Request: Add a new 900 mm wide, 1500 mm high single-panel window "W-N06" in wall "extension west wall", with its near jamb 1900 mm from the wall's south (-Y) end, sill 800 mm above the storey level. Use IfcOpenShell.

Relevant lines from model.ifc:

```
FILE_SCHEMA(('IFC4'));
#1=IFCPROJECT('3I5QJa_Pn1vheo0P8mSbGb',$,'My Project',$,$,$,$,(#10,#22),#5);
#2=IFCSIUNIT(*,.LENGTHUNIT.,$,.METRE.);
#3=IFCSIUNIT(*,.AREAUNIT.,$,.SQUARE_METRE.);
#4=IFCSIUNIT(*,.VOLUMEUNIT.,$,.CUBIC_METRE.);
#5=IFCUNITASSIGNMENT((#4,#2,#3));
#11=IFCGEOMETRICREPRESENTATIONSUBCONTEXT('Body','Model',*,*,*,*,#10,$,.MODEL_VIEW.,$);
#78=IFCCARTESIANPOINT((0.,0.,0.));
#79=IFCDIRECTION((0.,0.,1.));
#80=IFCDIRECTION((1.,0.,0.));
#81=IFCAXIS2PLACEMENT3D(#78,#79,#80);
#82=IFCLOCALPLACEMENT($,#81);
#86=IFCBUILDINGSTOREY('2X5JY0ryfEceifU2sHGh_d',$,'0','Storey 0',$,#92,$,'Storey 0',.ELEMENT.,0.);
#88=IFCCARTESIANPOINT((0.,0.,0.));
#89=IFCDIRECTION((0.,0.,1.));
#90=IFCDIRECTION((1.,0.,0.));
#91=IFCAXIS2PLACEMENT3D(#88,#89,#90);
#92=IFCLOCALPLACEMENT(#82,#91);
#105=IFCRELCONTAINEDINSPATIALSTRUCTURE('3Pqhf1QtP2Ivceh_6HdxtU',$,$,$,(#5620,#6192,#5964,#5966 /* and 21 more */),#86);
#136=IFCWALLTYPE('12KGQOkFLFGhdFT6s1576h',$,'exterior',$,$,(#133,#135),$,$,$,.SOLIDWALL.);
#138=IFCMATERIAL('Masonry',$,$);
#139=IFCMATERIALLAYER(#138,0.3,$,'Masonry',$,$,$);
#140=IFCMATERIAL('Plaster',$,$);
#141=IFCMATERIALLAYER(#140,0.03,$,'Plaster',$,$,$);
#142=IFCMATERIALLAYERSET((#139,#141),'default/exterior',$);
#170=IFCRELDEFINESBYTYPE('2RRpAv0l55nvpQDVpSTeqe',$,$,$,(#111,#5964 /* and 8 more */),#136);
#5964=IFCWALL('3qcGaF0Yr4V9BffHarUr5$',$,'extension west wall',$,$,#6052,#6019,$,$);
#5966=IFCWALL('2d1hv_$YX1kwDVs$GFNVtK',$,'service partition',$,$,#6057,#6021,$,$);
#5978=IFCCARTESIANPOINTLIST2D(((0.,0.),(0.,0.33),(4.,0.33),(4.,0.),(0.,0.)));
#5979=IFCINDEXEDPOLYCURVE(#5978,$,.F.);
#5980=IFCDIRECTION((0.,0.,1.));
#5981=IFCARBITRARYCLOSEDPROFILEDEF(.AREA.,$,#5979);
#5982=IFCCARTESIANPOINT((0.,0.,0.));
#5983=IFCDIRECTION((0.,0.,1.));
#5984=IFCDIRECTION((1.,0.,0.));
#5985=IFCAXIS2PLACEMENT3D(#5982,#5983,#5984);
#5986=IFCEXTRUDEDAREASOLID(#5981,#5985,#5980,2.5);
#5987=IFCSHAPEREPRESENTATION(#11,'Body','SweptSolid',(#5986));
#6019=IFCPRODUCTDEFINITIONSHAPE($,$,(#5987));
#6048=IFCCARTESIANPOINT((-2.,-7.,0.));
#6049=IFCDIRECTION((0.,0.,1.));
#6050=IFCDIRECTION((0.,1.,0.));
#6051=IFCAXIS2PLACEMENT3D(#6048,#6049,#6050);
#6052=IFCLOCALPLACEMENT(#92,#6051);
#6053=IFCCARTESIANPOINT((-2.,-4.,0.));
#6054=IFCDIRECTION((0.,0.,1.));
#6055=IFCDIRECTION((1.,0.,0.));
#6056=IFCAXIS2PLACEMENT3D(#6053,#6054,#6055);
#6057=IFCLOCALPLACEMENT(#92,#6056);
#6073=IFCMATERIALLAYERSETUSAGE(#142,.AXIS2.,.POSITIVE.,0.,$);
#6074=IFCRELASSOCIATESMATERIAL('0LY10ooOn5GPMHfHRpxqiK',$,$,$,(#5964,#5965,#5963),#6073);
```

```python
import numpy as np
import ifcopenshell
import ifcopenshell.api.feature
import ifcopenshell.api.geometry
import ifcopenshell.api.root
import ifcopenshell.api.spatial
import ifcopenshell.geom
import ifcopenshell.util.element
import ifcopenshell.util.placement
import ifcopenshell.util.representation
import ifcopenshell.util.shape
import ifcopenshell.util.unit

model = ifcopenshell.open("model.ifc")
unit_scale = ifcopenshell.util.unit.calculate_unit_scale(model)
settings = ifcopenshell.geom.settings()


def volume(element):
    """Net volume in cubic metres, openings subtracted."""
    shape = ifcopenshell.geom.create_shape(settings, element)
    return ifcopenshell.util.shape.get_volume(shape.geometry)


wall = model.by_guid("3qcGaF0Yr4V9BffHarUr5$")
storey = ifcopenshell.util.element.get_container(wall, ifc_class="IfcBuildingStorey")
context = ifcopenshell.util.representation.get_context(model, "Model", "Body", "MODEL_VIEW")
before = volume(wall)

width, height, from_end, sill = 0.9, 1.5, 1.9, 0.8  # metres

# The wall runs along its own X axis, and the end named is its -X end.
wall_shape = ifcopenshell.geom.create_shape(settings, wall)
x, y, z = ifcopenshell.util.shape.get_vertices(wall_shape.geometry).T
start = x.min() + from_end
face, thickness = float(y.min()), float(y.max() - y.min())
wall_matrix = ifcopenshell.util.placement.get_local_placement(wall.ObjectPlacement)
level = ifcopenshell.util.placement.get_local_placement(storey.ObjectPlacement)[2, 3]


def in_wall(x, y):
    """Placement at x, y metres in the wall's axes, at sill height."""
    matrix = wall_matrix.copy()
    matrix[:, 3] = wall_matrix @ np.array([x / unit_scale, y / unit_scale, 0.0, 1.0])
    matrix[2, 3] = level + sill / unit_scale
    return matrix


# Opening: a box that overshoots both wall faces by 50 mm.
opening = ifcopenshell.api.root.create_entity(model, ifc_class="IfcOpeningElement", predefined_type="OPENING")
box = ifcopenshell.api.geometry.add_wall_representation(
    model, context=context, length=width, height=height, thickness=thickness + 0.1
)
ifcopenshell.api.geometry.assign_representation(model, product=opening, representation=box)
ifcopenshell.api.geometry.edit_object_placement(model, product=opening, matrix=in_wall(start, face - 0.05), is_si=False)
ifcopenshell.api.feature.add_feature(model, feature=opening, element=wall)

window = ifcopenshell.api.root.create_entity(model, ifc_class="IfcWindow", name="W-N06", predefined_type="WINDOW")
window.OverallWidth, window.OverallHeight = width / unit_scale, height / unit_scale
window.PartitioningType = "SINGLE_PANEL"
body = ifcopenshell.api.geometry.add_window_representation(
    model,
    context=context,
    overall_width=window.OverallWidth,
    overall_height=window.OverallHeight,
    partition_type="SINGLE_PANEL",
)
ifcopenshell.api.geometry.assign_representation(model, product=window, representation=body)
ifcopenshell.api.spatial.assign_container(model, products=[window], relating_structure=storey)
ifcopenshell.api.feature.add_filling(model, opening=opening, element=window)

# Centre the window in the wall's thickness.
ifcopenshell.api.geometry.edit_object_placement(model, product=window, matrix=in_wall(start, face), is_si=False)
window_shape = ifcopenshell.geom.create_shape(settings, window)
depth = ifcopenshell.util.shape.get_vertices(window_shape.geometry)[:, 1]
offset = face + thickness / 2 - (depth.min() + depth.max()) / 2
ifcopenshell.api.geometry.edit_object_placement(model, product=window, matrix=in_wall(start, offset), is_si=False)

after = volume(wall)

print(f"wall volume {before:.3f} -> {after:.3f} m3")

model.write("model_edited.ifc")
```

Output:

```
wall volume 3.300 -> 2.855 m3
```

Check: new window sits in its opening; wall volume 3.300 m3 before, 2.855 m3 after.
